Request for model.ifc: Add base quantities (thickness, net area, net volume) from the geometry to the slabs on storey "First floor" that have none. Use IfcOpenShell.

First a look at what the model holds.

```python
import ifcopenshell
import ifcopenshell.util.element
import ifcopenshell.util.unit

model = ifcopenshell.open("model.ifc")
print(model.schema)
for unit_type in ("LENGTHUNIT", "AREAUNIT", "VOLUMEUNIT"):
    print(unit_type, ifcopenshell.util.unit.calculate_unit_scale(model, unit_type))
storey = next(s for s in model.by_type("IfcBuildingStorey") if s.Name == "First floor")
slabs = [e for e in ifcopenshell.util.element.get_decomposition(storey) if e.is_a("IfcSlab")]
for e in sorted(slabs, key=lambda e: e.id()):
    print(e.id(), e.is_a(), e.Name, list(ifcopenshell.util.element.get_psets(e, qtos_only=True)), sep=" | ")
```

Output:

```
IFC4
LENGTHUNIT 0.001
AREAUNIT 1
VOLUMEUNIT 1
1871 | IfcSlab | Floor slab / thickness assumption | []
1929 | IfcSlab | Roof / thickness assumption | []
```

```python
import ifcopenshell
import ifcopenshell.api.pset
import ifcopenshell.geom
import ifcopenshell.util.element
import ifcopenshell.util.shape
import ifcopenshell.util.unit

model = ifcopenshell.open("model.ifc")
unit_scale = ifcopenshell.util.unit.calculate_unit_scale(model)
area_scale = ifcopenshell.util.unit.calculate_unit_scale(model, "AREAUNIT")
volume_scale = ifcopenshell.util.unit.calculate_unit_scale(model, "VOLUMEUNIT")
settings = ifcopenshell.geom.settings()

storey = next(s for s in model.by_type("IfcBuildingStorey") if s.Name == "First floor")
slabs = [e for e in ifcopenshell.util.element.get_decomposition(storey) if e.is_a("IfcSlab")]

for e in sorted(slabs, key=lambda e: e.id()):
    if ifcopenshell.util.element.get_psets(e, qtos_only=True, should_inherit=False):
        continue
    # Geometry comes back in metres, in the element's own axes.
    shape = ifcopenshell.geom.create_shape(settings, e)
    values = {
        "Width": ifcopenshell.util.shape.get_z(shape.geometry) / unit_scale,
        "NetArea": ifcopenshell.util.shape.get_footprint_area(shape.geometry) / area_scale,
        "NetVolume": ifcopenshell.util.shape.get_volume(shape.geometry) / volume_scale,
    }
    qto = ifcopenshell.api.pset.add_qto(model, product=e, name="Qto_SlabBaseQuantities")
    ifcopenshell.api.pset.edit_qto(model, qto=qto, properties=values)
    print(e.id(), {k: round(v, 3) for k, v in values.items()})

model.write("model-out.ifc")
```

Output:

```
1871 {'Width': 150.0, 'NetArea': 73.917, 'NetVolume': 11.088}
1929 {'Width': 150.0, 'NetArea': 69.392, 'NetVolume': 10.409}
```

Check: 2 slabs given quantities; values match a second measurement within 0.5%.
